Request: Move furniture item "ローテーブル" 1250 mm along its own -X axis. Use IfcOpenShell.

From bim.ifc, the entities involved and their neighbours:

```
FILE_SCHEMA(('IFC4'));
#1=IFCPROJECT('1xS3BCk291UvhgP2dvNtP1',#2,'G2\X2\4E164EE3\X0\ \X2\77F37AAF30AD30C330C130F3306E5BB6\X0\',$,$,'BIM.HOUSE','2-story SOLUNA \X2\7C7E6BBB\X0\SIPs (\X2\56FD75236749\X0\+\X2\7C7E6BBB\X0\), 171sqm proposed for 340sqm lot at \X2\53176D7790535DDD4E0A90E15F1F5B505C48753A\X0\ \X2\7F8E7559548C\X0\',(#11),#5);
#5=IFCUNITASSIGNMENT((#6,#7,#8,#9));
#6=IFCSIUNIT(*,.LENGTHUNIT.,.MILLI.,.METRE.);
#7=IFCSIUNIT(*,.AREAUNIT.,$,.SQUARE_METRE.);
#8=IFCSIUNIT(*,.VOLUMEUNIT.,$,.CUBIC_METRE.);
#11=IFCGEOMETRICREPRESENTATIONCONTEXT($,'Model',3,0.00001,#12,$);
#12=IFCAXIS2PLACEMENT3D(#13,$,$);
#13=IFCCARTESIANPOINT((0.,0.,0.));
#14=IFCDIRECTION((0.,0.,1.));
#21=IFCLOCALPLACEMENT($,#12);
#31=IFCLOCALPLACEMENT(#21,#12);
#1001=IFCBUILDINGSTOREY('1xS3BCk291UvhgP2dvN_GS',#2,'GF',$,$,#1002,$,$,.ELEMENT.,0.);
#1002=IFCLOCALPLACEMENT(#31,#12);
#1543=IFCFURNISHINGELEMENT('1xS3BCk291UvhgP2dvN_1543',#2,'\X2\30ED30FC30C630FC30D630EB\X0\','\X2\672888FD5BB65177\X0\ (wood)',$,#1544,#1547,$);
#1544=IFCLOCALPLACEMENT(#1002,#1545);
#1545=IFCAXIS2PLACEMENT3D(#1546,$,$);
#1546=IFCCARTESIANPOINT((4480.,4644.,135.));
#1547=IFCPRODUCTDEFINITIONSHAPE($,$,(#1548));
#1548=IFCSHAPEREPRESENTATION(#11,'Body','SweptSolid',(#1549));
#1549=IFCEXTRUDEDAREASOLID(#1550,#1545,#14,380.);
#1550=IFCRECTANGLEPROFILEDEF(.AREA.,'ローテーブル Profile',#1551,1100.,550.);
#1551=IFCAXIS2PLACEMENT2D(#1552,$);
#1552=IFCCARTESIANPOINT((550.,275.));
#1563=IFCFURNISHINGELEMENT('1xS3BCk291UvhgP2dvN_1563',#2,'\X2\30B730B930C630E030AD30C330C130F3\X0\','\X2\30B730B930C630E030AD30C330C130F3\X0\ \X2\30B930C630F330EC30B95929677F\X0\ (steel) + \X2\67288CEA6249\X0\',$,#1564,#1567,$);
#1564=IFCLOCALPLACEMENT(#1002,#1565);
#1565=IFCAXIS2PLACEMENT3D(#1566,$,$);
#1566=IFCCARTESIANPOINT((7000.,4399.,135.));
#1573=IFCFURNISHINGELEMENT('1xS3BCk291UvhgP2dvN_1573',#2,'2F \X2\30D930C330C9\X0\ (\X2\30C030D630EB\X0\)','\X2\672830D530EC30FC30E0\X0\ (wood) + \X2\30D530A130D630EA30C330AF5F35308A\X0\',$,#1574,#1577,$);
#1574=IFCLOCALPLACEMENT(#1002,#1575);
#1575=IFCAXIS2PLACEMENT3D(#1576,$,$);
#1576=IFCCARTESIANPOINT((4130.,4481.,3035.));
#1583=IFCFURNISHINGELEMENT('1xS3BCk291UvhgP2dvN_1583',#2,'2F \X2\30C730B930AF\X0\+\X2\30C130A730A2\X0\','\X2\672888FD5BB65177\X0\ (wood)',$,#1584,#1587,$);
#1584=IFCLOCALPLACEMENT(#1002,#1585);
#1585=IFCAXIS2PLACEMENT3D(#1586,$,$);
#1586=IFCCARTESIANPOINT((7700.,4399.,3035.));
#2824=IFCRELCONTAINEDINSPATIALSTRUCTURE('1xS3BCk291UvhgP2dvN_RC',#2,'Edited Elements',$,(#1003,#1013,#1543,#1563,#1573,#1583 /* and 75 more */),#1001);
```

```python
import ifcopenshell
import ifcopenshell.api.geometry
import ifcopenshell.util.placement
import ifcopenshell.util.unit

model = ifcopenshell.open("bim.ifc")
unit_scale = ifcopenshell.util.unit.calculate_unit_scale(model)

item = model.by_guid("1xS3BCk291UvhgP2dvN_1543")
matrix = ifcopenshell.util.placement.get_local_placement(item.ObjectPlacement)
matrix[:3, 3] -= matrix[:3, 0] * 1.25 / unit_scale
ifcopenshell.api.geometry.edit_object_placement(model, product=item, matrix=matrix, is_si=False)

print(ifcopenshell.util.placement.get_local_placement(item.ObjectPlacement).round(3) + 0.0)

model.write("bim-out.ifc")
```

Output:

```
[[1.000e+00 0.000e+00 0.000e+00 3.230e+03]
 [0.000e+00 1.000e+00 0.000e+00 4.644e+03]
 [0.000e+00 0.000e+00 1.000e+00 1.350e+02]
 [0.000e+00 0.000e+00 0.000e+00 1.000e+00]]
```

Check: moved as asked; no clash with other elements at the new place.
